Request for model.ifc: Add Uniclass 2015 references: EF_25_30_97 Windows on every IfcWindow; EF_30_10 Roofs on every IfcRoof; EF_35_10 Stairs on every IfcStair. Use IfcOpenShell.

First a look at what the model holds.

```python
import ifcopenshell

model = ifcopenshell.open("model.ifc")
print(model.schema)
print("classifications:", [c.Name for c in model.by_type("IfcClassification")])
for ifc_class in ("IfcDoor", "IfcRoof", "IfcStair", "IfcWall", "IfcWindow"):
    print(ifc_class, len(model.by_type(ifc_class)))
```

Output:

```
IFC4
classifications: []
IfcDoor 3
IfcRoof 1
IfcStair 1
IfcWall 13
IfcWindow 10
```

```python
import ifcopenshell
import ifcopenshell.api.classification

model = ifcopenshell.open("model.ifc")

system = ifcopenshell.api.classification.add_classification(model, classification="Uniclass 2015")

codes = {
    "IfcWindow": ("EF_25_30_97", "Windows"),
    "IfcRoof": ("EF_30_10", "Roofs"),
    "IfcStair": ("EF_35_10", "Stairs"),
}
for ifc_class, (code, name) in codes.items():
    products = model.by_type(ifc_class)
    ifcopenshell.api.classification.add_reference(
        model, products=products, classification=system, identification=code, name=name
    )
    print(code, len(products))

model.write("model_updated.ifc")
```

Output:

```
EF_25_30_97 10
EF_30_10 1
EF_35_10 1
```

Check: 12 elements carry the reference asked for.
